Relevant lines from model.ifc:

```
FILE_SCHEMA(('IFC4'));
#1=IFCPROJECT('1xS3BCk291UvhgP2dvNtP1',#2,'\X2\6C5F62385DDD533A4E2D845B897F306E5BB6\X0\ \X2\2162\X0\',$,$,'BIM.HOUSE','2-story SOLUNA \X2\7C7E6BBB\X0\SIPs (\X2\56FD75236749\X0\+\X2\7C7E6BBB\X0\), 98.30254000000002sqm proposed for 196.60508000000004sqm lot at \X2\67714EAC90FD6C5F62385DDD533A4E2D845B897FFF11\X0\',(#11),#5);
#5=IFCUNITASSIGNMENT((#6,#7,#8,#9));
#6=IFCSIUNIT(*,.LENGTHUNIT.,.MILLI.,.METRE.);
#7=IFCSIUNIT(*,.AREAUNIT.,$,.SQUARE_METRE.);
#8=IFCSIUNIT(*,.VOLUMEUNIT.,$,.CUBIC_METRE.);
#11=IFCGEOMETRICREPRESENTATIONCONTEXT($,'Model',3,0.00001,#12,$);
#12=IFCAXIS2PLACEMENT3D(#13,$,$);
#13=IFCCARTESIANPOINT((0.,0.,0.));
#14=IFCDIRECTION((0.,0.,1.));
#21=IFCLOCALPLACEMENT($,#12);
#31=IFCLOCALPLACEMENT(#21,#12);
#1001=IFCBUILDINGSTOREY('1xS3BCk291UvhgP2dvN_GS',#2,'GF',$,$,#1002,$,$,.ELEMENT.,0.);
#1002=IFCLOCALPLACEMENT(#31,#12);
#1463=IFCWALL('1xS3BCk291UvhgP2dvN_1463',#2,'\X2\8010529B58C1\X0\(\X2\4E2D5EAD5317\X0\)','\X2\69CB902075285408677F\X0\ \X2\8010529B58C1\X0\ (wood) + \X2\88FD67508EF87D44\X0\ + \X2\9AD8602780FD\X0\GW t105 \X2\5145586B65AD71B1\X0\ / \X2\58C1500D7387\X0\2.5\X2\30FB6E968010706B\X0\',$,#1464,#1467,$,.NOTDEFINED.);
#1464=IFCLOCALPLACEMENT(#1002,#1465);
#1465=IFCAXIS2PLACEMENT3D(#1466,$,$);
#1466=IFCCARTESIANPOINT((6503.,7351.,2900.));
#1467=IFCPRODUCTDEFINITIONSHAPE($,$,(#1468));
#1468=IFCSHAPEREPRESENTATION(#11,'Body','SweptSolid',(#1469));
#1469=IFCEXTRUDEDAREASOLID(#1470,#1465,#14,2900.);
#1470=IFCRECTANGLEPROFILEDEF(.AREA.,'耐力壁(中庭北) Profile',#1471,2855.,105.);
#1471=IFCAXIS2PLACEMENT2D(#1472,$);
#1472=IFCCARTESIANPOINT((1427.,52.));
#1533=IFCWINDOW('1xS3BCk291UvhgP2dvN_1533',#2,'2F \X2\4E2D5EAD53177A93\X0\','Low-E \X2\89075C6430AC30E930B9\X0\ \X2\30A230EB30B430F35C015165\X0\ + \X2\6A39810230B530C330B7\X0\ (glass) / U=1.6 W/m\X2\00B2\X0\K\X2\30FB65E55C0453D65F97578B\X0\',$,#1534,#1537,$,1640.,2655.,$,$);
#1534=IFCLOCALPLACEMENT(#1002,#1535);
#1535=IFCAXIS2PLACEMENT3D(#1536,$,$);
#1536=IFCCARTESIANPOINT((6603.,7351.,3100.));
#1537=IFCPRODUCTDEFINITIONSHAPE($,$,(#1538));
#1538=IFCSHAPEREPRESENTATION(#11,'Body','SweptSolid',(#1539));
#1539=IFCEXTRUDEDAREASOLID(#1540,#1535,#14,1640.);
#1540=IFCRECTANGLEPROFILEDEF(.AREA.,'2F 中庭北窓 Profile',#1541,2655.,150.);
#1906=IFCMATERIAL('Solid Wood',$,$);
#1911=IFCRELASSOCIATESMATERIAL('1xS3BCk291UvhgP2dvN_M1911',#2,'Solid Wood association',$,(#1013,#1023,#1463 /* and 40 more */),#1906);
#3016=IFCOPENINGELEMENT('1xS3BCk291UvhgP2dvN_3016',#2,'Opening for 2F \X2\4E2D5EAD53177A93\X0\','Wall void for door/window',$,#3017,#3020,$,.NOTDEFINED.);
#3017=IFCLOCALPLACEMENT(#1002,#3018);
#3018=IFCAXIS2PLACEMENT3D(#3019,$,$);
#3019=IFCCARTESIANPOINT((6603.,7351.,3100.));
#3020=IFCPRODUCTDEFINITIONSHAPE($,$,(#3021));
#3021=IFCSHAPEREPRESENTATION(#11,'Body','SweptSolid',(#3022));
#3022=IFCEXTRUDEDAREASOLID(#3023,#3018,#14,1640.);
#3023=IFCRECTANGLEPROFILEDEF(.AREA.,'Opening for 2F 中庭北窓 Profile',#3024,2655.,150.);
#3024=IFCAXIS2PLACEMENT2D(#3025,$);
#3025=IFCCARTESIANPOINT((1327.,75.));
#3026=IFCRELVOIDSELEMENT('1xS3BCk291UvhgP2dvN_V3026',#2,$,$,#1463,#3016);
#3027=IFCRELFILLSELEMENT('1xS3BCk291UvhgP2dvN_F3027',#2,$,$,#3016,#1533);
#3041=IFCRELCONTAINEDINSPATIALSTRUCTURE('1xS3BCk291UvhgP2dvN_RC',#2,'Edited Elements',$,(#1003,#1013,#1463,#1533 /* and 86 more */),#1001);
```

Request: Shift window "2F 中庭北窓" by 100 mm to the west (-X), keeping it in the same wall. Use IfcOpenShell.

```python
import ifcopenshell
import ifcopenshell.api.geometry
import ifcopenshell.util.placement
import ifcopenshell.util.unit

model = ifcopenshell.open("model.ifc")
unit_scale = ifcopenshell.util.unit.calculate_unit_scale(model)

window = model.by_guid("1xS3BCk291UvhgP2dvN_1533")
opening = window.FillsVoids[0].RelatingOpeningElement
wall = opening.VoidsElements[0].RelatingBuildingElement

wall_matrix = ifcopenshell.util.placement.get_local_placement(wall.ObjectPlacement)
shift = wall_matrix[:3, 0] * -0.1 / unit_scale
before = ifcopenshell.util.placement.get_local_placement(window.ObjectPlacement)[:3, 3].copy()

# The window is not placed relative to its opening, so move both.
for product in (opening, window):
    matrix = ifcopenshell.util.placement.get_local_placement(product.ObjectPlacement)
    matrix[:3, 3] += shift
    ifcopenshell.api.geometry.edit_object_placement(model, product=product, matrix=matrix, is_si=False)

after = ifcopenshell.util.placement.get_local_placement(window.ObjectPlacement)[:3, 3]
print("window moved by", (after - before).round(3) + 0.0)

model.write("model_edited.ifc")
```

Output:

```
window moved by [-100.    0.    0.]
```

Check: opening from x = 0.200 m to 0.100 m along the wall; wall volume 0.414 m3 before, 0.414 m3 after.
